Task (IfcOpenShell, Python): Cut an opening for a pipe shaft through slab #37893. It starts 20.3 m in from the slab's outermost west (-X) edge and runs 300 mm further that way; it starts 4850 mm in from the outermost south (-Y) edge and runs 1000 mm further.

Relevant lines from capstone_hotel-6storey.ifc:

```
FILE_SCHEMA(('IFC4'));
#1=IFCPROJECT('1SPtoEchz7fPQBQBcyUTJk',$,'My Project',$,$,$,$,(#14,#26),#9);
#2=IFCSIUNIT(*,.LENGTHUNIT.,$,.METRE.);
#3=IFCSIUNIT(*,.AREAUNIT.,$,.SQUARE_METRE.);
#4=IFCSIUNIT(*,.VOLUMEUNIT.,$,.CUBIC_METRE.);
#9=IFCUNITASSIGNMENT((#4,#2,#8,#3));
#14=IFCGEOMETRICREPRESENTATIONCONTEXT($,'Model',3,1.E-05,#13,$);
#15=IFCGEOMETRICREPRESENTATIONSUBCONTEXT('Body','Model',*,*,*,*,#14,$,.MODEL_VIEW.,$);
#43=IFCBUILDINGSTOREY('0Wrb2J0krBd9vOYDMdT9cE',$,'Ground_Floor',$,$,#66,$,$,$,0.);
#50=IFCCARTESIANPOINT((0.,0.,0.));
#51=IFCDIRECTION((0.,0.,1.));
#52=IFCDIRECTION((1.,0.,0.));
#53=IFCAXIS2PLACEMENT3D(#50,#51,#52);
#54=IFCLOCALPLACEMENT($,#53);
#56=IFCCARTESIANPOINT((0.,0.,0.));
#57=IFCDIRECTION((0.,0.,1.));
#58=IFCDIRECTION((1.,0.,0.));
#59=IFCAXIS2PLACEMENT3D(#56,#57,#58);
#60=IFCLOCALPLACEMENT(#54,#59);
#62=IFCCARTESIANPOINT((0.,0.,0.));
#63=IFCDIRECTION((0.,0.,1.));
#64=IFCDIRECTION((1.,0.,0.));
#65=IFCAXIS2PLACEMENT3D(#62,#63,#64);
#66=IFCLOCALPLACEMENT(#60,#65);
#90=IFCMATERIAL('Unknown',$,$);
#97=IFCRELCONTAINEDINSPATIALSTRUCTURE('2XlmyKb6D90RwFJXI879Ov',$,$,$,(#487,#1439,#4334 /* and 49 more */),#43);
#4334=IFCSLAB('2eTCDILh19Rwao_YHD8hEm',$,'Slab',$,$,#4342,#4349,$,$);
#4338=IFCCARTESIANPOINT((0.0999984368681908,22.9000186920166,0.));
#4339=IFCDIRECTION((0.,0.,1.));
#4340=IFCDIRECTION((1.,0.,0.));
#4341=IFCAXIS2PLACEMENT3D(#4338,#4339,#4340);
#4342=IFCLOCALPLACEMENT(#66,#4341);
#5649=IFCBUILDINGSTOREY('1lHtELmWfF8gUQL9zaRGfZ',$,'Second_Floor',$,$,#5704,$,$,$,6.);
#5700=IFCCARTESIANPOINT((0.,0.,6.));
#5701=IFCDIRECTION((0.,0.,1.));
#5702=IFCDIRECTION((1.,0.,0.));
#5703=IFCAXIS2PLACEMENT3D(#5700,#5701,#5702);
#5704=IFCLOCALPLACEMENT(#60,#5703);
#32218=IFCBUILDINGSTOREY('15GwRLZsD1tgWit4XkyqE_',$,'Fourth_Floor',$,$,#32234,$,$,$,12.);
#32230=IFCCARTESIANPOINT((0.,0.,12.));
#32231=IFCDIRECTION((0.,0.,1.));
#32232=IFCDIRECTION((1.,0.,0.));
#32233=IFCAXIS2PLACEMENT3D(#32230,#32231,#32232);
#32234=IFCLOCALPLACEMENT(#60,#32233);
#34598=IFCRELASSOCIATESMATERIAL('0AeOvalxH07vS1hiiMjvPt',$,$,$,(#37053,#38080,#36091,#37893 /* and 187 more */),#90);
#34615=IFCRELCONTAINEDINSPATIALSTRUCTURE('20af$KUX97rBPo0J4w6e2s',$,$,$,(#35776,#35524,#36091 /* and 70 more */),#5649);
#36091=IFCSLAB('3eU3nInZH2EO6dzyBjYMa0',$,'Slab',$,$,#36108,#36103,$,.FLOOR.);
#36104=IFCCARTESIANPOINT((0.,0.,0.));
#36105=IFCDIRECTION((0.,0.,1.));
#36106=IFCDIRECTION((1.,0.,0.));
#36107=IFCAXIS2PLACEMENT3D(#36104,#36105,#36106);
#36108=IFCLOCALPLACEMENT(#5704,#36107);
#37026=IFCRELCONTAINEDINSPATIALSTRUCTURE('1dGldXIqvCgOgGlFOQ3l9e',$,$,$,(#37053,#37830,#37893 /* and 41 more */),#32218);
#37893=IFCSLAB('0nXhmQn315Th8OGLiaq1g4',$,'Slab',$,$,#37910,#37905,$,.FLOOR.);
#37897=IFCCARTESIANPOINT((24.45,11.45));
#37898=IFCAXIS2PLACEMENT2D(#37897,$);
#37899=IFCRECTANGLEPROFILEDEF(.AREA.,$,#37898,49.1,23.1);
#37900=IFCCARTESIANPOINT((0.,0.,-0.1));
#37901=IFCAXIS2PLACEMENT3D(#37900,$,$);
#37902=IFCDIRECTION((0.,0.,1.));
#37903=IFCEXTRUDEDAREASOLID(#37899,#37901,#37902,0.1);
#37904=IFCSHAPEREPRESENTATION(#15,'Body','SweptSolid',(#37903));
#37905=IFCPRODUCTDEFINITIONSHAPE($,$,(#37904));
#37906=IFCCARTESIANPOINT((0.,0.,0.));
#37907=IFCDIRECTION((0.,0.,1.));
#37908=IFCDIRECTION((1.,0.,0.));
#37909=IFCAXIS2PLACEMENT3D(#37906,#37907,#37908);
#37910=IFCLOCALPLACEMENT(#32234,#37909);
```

```python
import numpy as np
import ifcopenshell
import ifcopenshell.api.feature
import ifcopenshell.api.geometry
import ifcopenshell.api.root
import ifcopenshell.geom
import ifcopenshell.util.placement
import ifcopenshell.util.representation
import ifcopenshell.util.shape
import ifcopenshell.util.unit

model = ifcopenshell.open("capstone_hotel-6storey.ifc")
unit_scale = ifcopenshell.util.unit.calculate_unit_scale(model)
settings = ifcopenshell.geom.settings()


def volume(element):
    """Net volume in cubic metres, openings subtracted."""
    shape = ifcopenshell.geom.create_shape(settings, element)
    return ifcopenshell.util.shape.get_volume(shape.geometry)


slab = model.by_guid("0nXhmQn315Th8OGLiaq1g4")
before = volume(slab)

# Extent in the slab's own axes, in metres. The edges named are its -X and -Y sides.
slab_shape = ifcopenshell.geom.create_shape(settings, slab)
vertices = ifcopenshell.util.shape.get_vertices(slab_shape.geometry)
x_min, y_min, bottom = vertices.min(axis=0)
top = vertices[:, 2].max()

opening = ifcopenshell.api.root.create_entity(model, ifc_class="IfcOpeningElement", name="Pipe shaft opening", predefined_type="OPENING")
context = ifcopenshell.util.representation.get_context(model, "Model", "Body", "MODEL_VIEW")
width, depth = 0.3, 1
outline = [(0.0, 0.0), (width, 0.0), (width, depth), (0.0, depth), (0.0, 0.0)]
# Overshoot both faces by 50 mm so the cut is clean.
shape = ifcopenshell.api.geometry.add_slab_representation(
    model, context=context, depth=top - bottom + 0.1, polyline=outline
)
ifcopenshell.api.geometry.assign_representation(model, product=opening, representation=shape)

matrix = ifcopenshell.util.placement.get_local_placement(slab.ObjectPlacement)
matrix[:, 3] = matrix @ np.append(np.array([x_min + 20.3, y_min + 4.85, bottom - 0.05]) / unit_scale, 1.0)
ifcopenshell.api.geometry.edit_object_placement(model, product=opening, matrix=matrix, is_si=False)
ifcopenshell.api.feature.add_feature(model, feature=opening, element=slab)

after = volume(slab)

print(f"slab volume {before:.3f} -> {after:.3f} m3")

model.write("capstone_hotel-6storey_v2.ifc")
```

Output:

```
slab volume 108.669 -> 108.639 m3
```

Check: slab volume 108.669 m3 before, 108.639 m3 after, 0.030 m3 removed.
